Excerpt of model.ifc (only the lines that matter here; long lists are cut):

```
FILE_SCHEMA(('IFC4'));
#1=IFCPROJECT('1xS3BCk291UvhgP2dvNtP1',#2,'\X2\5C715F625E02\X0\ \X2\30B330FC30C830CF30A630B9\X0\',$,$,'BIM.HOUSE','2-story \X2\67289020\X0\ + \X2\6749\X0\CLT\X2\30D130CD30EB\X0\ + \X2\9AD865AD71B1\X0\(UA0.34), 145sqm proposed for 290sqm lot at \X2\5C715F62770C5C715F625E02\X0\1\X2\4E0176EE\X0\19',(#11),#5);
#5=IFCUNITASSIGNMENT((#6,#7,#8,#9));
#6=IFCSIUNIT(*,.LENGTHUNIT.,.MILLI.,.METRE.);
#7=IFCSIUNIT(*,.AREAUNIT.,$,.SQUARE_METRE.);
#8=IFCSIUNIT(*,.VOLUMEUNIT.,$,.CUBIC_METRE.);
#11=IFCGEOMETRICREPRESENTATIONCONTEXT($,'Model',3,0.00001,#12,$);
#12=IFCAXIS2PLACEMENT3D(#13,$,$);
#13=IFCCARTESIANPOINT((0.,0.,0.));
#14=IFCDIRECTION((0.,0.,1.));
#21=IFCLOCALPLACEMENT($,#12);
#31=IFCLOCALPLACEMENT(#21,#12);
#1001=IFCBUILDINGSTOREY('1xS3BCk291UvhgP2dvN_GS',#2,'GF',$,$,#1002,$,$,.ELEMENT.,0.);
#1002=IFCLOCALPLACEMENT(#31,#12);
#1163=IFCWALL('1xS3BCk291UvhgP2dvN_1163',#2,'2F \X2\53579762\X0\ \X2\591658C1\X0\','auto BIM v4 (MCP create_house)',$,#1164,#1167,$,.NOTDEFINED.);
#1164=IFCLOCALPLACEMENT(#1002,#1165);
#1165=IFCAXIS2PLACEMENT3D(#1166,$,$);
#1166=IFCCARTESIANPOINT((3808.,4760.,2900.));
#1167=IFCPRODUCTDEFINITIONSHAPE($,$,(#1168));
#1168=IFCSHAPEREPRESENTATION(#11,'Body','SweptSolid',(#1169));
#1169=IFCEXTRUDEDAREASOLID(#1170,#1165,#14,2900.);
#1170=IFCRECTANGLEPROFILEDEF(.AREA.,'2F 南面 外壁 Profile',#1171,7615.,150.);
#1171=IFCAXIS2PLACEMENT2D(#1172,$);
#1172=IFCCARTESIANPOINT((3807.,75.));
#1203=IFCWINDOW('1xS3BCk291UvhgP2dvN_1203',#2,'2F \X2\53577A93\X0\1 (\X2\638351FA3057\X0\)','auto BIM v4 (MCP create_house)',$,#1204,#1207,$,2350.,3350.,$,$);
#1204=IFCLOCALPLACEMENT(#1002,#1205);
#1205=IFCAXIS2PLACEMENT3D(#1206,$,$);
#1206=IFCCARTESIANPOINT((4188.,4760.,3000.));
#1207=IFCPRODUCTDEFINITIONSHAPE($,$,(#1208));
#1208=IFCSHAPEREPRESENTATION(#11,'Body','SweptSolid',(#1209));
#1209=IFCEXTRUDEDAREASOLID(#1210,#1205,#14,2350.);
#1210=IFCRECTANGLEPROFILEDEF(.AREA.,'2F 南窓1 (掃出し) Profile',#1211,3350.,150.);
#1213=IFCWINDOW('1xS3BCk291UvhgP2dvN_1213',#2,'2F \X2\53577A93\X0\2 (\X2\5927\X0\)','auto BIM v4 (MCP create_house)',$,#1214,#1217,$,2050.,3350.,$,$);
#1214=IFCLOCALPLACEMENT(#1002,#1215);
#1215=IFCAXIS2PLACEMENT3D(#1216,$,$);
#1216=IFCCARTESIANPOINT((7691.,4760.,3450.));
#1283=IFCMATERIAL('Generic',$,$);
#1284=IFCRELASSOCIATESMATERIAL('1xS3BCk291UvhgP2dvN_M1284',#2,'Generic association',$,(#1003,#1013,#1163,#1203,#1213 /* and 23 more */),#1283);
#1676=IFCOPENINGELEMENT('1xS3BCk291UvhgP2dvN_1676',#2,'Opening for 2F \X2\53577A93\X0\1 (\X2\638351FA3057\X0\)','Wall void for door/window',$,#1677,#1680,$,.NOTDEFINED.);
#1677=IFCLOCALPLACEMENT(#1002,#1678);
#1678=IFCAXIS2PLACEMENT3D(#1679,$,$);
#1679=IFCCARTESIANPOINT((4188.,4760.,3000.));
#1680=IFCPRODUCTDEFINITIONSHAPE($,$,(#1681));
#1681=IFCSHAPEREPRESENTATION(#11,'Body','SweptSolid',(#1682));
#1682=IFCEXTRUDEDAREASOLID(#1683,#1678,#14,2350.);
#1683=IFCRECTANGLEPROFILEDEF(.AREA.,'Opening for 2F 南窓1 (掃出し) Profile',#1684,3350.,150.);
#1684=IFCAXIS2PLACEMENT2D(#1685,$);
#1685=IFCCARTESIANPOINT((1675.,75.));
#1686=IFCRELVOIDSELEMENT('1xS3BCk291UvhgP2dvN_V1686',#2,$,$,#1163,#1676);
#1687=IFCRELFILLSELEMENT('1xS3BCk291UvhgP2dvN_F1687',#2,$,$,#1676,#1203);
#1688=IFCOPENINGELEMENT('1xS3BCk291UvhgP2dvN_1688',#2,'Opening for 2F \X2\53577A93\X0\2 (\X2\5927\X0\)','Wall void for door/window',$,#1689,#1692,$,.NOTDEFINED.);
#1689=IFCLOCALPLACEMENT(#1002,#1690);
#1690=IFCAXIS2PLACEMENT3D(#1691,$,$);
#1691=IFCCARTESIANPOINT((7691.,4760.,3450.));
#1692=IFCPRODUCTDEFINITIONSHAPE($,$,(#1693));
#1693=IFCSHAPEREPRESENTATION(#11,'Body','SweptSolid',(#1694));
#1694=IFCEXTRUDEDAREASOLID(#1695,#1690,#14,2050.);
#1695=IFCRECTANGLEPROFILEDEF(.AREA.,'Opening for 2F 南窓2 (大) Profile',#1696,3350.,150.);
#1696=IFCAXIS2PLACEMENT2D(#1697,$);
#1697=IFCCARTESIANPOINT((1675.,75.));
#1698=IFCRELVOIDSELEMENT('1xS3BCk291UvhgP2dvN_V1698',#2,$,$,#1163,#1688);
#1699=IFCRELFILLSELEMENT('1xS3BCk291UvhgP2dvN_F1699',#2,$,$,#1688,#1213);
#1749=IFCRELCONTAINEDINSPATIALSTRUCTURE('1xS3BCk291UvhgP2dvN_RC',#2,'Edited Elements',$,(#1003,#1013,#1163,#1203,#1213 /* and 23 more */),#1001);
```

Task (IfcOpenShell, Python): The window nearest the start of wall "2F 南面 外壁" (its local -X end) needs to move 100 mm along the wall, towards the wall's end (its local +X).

```python
import ifcopenshell
import ifcopenshell.api.geometry
import ifcopenshell.util.placement
import ifcopenshell.util.unit

model = ifcopenshell.open("model.ifc")
unit_scale = ifcopenshell.util.unit.calculate_unit_scale(model)

window = model.by_guid("1xS3BCk291UvhgP2dvN_1203")
opening = window.FillsVoids[0].RelatingOpeningElement
wall = opening.VoidsElements[0].RelatingBuildingElement

wall_matrix = ifcopenshell.util.placement.get_local_placement(wall.ObjectPlacement)
shift = wall_matrix[:3, 0] * 0.1 / unit_scale
before = ifcopenshell.util.placement.get_local_placement(window.ObjectPlacement)[:3, 3].copy()

# The window is not placed relative to its opening, so move both.
for product in (opening, window):
    matrix = ifcopenshell.util.placement.get_local_placement(product.ObjectPlacement)
    matrix[:3, 3] += shift
    ifcopenshell.api.geometry.edit_object_placement(model, product=product, matrix=matrix, is_si=False)

after = ifcopenshell.util.placement.get_local_placement(window.ObjectPlacement)[:3, 3]
print("window moved by", (after - before).round(3) + 0.0)

model.write("model_edited.ifc")
```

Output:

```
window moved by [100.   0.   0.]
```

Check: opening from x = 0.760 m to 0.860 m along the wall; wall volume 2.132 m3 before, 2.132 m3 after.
